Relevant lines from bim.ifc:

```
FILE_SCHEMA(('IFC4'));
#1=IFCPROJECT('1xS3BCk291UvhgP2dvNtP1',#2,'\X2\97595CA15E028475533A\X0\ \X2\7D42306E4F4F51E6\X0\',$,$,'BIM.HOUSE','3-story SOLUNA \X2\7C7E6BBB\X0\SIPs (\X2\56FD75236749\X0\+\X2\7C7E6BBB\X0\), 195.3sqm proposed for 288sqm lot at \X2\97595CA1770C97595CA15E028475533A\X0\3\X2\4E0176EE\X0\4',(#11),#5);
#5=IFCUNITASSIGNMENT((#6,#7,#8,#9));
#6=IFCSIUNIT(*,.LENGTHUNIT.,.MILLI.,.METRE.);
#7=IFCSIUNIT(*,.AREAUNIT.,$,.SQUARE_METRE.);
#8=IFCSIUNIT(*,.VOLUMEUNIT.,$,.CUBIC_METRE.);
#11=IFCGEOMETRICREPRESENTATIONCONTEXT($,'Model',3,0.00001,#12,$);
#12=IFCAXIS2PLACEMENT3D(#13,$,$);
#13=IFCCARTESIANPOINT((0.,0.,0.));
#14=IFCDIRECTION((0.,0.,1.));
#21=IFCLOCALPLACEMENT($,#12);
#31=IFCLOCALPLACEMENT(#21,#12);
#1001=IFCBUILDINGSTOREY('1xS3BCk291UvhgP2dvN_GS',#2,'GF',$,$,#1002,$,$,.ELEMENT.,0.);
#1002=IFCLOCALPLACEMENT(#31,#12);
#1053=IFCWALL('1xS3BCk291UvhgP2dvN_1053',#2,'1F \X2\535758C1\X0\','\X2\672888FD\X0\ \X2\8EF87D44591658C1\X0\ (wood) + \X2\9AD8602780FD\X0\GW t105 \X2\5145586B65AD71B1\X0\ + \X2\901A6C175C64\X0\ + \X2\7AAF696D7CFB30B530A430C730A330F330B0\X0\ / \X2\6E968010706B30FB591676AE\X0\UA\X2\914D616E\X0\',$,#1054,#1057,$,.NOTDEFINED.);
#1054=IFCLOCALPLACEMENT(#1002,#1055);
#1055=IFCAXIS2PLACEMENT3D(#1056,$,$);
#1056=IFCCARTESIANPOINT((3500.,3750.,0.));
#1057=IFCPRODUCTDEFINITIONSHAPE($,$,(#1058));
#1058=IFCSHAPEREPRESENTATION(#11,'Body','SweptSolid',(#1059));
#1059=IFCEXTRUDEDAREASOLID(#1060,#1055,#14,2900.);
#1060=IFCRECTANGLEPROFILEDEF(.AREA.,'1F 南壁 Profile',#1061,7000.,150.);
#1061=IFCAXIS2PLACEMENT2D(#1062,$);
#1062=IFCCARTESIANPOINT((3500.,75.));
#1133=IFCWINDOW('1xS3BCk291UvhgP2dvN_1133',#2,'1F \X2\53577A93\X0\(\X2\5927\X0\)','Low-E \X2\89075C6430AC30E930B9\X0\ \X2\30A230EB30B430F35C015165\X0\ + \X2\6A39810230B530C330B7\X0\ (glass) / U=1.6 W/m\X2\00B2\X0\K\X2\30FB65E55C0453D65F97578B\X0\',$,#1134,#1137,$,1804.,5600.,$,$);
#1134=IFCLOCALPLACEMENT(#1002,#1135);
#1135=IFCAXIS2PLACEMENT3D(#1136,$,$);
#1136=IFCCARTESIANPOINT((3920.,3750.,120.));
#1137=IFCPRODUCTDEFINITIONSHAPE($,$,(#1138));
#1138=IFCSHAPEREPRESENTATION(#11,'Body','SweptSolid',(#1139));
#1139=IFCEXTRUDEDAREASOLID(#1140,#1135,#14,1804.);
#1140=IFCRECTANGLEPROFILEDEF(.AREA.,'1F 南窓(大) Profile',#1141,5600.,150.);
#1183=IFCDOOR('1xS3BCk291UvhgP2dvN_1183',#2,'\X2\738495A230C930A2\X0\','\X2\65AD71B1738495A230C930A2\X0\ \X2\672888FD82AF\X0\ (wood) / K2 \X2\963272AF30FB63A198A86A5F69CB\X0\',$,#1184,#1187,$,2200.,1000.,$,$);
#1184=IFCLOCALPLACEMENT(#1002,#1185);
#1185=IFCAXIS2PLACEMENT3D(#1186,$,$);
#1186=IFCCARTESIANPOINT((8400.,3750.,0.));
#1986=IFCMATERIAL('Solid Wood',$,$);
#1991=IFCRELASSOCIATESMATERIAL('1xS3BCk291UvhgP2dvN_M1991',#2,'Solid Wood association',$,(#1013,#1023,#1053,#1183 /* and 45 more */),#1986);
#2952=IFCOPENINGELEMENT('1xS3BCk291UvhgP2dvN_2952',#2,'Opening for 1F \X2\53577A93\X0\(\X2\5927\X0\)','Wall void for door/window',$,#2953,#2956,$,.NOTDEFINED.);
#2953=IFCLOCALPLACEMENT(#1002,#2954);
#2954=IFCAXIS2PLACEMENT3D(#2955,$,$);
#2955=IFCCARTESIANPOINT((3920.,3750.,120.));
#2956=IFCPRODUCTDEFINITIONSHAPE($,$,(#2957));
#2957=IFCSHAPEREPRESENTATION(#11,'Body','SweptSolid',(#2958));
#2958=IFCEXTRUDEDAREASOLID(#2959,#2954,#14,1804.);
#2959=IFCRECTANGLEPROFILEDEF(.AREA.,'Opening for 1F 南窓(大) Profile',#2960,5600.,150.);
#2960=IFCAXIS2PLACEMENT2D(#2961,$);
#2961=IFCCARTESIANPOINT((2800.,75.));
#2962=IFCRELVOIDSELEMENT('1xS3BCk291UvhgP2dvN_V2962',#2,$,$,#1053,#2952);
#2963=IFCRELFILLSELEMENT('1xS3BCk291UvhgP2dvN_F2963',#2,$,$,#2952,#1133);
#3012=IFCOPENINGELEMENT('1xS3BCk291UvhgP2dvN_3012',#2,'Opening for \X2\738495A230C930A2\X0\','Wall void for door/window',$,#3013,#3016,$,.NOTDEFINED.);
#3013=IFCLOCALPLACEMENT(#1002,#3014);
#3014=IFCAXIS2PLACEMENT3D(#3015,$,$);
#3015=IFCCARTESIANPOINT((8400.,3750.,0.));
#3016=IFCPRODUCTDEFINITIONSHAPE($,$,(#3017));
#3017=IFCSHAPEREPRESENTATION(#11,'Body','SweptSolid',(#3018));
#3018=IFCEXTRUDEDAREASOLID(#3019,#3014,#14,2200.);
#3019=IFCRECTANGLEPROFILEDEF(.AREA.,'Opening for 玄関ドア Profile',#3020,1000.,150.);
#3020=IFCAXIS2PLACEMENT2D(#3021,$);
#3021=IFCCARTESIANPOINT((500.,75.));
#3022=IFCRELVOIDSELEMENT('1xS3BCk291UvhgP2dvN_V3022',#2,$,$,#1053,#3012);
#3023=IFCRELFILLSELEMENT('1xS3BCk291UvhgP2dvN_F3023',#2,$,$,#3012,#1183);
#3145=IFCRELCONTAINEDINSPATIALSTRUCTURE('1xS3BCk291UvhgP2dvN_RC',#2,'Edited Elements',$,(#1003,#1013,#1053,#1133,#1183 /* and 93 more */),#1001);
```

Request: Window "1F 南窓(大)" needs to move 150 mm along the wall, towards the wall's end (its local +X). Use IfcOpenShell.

```python
import ifcopenshell
import ifcopenshell.api.geometry
import ifcopenshell.util.placement

model = ifcopenshell.open("bim.ifc")

window = model.by_id(1133)
opening = window.FillsVoids[0].RelatingOpeningElement
wall = opening.VoidsElements[0].RelatingBuildingElement

wall_matrix = ifcopenshell.util.placement.get_local_placement(wall.ObjectPlacement)
shift = wall_matrix[:3, 0] * 150.0
before = ifcopenshell.util.placement.get_local_placement(window.ObjectPlacement)[:3, 3].copy()

# The window is not placed relative to its opening, so move both.
for product in (opening, window):
    matrix = ifcopenshell.util.placement.get_local_placement(product.ObjectPlacement)
    matrix[:3, 3] += shift
    ifcopenshell.api.geometry.edit_object_placement(model, product=product, matrix=matrix, is_si=False)

after = ifcopenshell.util.placement.get_local_placement(window.ObjectPlacement)[:3, 3]
print("window moved by", (after - before).round(3) + 0.0)

model.write("bim_v2.ifc")
```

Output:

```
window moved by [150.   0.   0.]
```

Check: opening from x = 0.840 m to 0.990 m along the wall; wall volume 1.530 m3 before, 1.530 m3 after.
